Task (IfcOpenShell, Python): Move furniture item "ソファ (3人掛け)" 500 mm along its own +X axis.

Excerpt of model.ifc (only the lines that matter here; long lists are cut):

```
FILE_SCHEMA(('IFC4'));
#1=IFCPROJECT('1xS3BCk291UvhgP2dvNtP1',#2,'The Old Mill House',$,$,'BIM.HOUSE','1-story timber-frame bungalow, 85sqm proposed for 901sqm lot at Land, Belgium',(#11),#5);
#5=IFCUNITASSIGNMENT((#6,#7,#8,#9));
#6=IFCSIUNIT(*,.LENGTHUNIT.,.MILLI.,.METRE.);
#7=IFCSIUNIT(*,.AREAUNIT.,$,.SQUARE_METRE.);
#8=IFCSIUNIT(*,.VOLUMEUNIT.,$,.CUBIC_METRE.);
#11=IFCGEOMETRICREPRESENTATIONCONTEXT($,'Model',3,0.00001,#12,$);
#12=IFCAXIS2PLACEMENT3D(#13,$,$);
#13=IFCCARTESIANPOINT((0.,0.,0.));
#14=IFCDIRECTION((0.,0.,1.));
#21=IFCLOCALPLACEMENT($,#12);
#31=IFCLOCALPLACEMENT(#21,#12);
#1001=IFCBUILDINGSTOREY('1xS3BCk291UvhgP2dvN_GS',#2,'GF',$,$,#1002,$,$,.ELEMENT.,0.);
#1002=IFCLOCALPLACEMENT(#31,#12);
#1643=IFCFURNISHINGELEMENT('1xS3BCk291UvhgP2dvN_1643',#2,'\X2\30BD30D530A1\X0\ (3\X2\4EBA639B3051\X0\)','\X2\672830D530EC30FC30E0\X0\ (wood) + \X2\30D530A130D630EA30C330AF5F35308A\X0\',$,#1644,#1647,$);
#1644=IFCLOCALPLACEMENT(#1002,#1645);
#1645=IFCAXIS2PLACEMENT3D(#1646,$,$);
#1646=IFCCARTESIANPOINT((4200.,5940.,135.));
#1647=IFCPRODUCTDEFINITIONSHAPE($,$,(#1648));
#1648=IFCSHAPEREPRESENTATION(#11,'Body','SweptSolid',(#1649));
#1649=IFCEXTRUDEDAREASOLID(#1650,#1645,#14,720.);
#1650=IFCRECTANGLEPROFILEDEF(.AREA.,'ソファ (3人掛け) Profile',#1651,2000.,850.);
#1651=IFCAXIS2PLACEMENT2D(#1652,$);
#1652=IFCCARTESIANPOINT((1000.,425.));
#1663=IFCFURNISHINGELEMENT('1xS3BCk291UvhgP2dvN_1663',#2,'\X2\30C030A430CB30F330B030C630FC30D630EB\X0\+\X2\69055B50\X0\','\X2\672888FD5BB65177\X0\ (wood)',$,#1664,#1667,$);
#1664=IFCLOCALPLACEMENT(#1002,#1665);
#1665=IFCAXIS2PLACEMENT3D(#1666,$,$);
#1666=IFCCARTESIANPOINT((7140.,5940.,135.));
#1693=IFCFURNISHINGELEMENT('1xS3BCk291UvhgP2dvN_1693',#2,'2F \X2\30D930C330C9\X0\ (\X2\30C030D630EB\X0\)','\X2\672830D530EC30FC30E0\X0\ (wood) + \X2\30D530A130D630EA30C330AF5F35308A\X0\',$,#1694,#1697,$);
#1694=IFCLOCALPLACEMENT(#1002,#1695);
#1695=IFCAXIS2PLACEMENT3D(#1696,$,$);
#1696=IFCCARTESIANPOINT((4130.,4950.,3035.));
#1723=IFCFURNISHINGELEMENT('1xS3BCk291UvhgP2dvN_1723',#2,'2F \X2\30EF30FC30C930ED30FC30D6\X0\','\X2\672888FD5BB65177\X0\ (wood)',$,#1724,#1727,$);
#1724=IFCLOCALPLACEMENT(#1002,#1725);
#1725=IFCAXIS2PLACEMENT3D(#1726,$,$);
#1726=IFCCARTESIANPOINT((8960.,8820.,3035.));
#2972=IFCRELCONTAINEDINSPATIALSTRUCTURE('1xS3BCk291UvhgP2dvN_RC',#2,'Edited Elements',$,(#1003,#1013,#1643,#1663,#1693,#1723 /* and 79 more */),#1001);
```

```python
import ifcopenshell
import ifcopenshell.api.geometry
import ifcopenshell.util.placement

model = ifcopenshell.open("model.ifc")

item = model.by_id(1643)
matrix = ifcopenshell.util.placement.get_local_placement(item.ObjectPlacement)
matrix[:3, 3] += matrix[:3, 0] * 500.0
ifcopenshell.api.geometry.edit_object_placement(model, product=item, matrix=matrix, is_si=False)

print(ifcopenshell.util.placement.get_local_placement(item.ObjectPlacement).round(3) + 0.0)

model.write("model-out.ifc")
```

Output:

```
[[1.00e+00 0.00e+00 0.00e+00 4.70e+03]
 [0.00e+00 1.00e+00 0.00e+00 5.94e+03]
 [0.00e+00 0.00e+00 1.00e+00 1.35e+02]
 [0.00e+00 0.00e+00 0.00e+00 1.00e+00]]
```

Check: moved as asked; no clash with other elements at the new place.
